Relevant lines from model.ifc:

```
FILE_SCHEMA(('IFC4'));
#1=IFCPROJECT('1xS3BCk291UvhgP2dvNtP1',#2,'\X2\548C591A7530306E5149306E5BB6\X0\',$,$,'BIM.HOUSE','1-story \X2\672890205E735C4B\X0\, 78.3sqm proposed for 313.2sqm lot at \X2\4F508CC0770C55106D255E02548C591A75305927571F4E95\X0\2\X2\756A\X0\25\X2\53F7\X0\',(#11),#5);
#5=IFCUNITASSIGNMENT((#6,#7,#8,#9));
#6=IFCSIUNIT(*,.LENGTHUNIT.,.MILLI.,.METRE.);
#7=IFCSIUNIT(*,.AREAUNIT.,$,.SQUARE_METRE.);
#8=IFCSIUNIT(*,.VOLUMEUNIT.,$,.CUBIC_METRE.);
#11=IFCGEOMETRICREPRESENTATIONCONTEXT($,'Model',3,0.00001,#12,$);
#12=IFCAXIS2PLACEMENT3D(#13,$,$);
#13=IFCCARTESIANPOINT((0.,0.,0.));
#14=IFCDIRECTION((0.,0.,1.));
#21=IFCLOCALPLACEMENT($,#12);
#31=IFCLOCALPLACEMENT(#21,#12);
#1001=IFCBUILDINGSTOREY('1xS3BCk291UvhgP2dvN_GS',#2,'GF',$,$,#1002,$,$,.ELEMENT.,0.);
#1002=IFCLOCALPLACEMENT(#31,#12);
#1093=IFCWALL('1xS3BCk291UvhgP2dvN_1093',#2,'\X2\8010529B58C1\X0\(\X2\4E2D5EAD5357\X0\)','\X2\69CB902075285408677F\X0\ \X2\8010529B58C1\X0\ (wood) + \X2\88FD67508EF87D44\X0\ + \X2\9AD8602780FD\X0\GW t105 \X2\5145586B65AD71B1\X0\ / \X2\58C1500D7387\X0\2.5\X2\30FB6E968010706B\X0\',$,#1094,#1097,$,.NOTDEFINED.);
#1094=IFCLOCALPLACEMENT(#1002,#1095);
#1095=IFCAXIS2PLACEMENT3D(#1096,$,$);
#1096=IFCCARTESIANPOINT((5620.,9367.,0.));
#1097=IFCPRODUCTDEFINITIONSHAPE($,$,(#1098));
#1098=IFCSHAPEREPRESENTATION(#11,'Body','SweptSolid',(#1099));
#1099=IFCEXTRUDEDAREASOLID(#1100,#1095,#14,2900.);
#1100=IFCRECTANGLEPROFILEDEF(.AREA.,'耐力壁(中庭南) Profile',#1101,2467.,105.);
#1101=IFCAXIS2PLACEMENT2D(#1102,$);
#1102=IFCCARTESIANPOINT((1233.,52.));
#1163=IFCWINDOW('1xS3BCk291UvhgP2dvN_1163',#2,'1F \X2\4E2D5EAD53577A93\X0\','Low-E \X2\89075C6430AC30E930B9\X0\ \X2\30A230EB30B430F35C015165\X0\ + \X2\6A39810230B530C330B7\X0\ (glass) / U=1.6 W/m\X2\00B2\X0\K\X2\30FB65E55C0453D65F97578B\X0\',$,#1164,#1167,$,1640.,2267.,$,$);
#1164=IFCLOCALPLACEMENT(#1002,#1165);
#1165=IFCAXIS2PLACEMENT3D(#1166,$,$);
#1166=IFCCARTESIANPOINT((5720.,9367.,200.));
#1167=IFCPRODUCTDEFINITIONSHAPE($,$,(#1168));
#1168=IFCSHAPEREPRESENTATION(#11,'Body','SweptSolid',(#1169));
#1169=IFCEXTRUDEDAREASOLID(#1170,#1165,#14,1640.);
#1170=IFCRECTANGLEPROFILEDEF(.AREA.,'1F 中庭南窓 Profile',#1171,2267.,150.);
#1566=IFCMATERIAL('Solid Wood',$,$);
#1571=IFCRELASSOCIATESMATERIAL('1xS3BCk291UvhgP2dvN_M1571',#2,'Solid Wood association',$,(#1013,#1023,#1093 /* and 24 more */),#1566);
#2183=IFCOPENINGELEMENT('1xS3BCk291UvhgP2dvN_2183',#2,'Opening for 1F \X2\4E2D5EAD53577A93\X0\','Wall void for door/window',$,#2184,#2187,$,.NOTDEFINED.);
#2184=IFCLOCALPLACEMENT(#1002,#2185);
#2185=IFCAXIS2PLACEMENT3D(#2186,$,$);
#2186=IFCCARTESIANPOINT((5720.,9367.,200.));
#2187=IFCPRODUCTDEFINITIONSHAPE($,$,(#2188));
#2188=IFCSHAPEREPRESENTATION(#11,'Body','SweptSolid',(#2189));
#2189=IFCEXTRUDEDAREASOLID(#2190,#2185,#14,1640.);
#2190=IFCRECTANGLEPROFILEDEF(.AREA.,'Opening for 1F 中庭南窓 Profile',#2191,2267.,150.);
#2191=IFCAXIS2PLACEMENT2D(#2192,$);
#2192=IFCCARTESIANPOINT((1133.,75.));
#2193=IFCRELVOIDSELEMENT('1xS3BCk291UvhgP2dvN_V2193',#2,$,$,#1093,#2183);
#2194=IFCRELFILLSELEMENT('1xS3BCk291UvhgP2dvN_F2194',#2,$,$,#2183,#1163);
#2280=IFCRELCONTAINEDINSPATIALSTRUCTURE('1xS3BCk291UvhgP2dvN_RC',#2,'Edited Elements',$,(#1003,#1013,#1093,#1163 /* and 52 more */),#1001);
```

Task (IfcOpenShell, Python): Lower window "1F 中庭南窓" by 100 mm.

```python
import numpy as np
import ifcopenshell
import ifcopenshell.api.geometry
import ifcopenshell.util.placement
import ifcopenshell.util.unit

model = ifcopenshell.open("model.ifc")
unit_scale = ifcopenshell.util.unit.calculate_unit_scale(model)

window = model.by_guid("1xS3BCk291UvhgP2dvN_1163")
opening = window.FillsVoids[0].RelatingOpeningElement
dz = -0.1 / unit_scale

shift = np.array([0.0, 0.0, dz])
# The window is not placed relative to its opening, so move both.
for product in (opening, window):
    matrix = ifcopenshell.util.placement.get_local_placement(product.ObjectPlacement)
    matrix[:3, 3] += shift
    ifcopenshell.api.geometry.edit_object_placement(model, product=product, matrix=matrix, is_si=False)

print(f"moved by {dz * unit_scale:+.3f} m")

model.write("model_v2.ifc")
```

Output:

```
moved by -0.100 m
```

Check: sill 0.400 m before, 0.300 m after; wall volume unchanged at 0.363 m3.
